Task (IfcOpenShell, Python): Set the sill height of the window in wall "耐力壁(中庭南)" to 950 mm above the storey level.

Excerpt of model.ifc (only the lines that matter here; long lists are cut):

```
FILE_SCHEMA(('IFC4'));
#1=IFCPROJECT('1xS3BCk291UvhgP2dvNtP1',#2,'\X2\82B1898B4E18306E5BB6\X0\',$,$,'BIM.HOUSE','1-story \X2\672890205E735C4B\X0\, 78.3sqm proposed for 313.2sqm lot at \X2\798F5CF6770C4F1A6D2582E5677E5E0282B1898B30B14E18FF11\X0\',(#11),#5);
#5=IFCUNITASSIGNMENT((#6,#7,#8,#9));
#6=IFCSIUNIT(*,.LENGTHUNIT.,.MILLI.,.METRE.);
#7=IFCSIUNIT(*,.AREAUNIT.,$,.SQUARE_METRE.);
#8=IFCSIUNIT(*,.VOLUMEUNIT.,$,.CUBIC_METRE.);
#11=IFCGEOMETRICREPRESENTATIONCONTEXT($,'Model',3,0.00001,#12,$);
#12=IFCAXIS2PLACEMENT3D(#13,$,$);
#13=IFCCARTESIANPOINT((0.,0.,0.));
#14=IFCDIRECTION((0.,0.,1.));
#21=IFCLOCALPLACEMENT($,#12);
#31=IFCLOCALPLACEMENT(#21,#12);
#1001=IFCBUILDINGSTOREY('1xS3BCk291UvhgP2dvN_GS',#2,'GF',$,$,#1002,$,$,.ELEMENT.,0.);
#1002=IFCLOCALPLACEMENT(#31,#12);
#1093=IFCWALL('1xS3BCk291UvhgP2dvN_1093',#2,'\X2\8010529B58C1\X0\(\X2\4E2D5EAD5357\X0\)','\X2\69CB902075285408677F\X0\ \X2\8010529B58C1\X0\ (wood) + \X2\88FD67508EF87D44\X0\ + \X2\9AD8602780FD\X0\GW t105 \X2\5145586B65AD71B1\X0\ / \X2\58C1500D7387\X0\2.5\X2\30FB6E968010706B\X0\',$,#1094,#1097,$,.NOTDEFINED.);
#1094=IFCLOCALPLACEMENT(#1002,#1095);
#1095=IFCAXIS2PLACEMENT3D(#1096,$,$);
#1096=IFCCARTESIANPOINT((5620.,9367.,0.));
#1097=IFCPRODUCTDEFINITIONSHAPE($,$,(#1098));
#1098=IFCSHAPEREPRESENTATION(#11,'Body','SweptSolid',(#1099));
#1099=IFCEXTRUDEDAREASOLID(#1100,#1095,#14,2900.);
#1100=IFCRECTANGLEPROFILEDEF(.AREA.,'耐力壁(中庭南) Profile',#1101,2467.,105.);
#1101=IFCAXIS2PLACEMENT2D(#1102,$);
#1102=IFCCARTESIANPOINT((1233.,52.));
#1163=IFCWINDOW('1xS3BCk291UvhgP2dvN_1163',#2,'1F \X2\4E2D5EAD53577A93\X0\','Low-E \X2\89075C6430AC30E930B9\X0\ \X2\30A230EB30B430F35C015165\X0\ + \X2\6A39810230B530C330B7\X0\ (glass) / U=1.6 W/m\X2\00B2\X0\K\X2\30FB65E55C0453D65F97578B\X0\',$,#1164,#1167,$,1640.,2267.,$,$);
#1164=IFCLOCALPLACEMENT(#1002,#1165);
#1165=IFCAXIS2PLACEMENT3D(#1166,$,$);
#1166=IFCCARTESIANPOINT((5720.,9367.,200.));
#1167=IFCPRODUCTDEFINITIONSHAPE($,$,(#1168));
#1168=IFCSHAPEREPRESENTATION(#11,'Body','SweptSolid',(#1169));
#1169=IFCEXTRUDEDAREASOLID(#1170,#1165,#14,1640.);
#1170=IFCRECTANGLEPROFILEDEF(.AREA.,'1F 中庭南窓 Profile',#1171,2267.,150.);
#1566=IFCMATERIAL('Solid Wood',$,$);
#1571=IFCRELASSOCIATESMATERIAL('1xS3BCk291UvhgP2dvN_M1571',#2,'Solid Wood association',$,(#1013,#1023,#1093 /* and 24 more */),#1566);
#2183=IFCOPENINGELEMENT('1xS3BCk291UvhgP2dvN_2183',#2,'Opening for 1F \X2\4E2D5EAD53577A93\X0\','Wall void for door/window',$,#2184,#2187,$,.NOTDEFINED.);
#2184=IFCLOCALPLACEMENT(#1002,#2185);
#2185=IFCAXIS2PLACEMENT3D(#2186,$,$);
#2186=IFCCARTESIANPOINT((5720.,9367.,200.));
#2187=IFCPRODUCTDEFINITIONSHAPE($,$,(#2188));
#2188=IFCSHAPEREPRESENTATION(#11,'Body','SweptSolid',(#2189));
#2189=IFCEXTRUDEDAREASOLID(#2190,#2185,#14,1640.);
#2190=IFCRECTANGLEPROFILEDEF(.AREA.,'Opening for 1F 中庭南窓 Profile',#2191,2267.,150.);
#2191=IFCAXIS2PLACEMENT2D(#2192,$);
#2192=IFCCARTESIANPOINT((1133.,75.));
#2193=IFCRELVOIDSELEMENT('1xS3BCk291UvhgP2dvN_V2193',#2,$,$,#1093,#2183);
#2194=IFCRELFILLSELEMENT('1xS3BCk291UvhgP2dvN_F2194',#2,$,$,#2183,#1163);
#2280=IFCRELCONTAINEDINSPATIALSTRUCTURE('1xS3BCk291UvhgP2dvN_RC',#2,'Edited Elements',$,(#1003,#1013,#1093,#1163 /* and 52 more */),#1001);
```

```python
import numpy as np
import ifcopenshell
import ifcopenshell.api.geometry
import ifcopenshell.geom
import ifcopenshell.util.element
import ifcopenshell.util.placement
import ifcopenshell.util.shape
import ifcopenshell.util.unit

model = ifcopenshell.open("model.ifc")
unit_scale = ifcopenshell.util.unit.calculate_unit_scale(model)

window = model.by_id(1163)
opening = window.FillsVoids[0].RelatingOpeningElement
storey = ifcopenshell.util.element.get_container(window, ifc_class="IfcBuildingStorey")
level = ifcopenshell.util.placement.get_local_placement(storey.ObjectPlacement)[2, 3]

# The opening's origin need not be at the sill, so measure its lowest point.
shape = ifcopenshell.geom.create_shape(ifcopenshell.geom.settings(), opening)
bottom = ifcopenshell.util.shape.get_shape_bottom_elevation(shape, shape.geometry) / unit_scale
dz = level + 0.95 / unit_scale - bottom

shift = np.array([0.0, 0.0, dz])
# The window is not placed relative to its opening, so move both.
for product in (opening, window):
    matrix = ifcopenshell.util.placement.get_local_placement(product.ObjectPlacement)
    matrix[:3, 3] += shift
    ifcopenshell.api.geometry.edit_object_placement(model, product=product, matrix=matrix, is_si=False)

print(f"moved by {dz * unit_scale:+.3f} m")

model.write("model_rev.ifc")
```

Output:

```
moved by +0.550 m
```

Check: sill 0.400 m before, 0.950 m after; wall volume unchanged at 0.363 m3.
